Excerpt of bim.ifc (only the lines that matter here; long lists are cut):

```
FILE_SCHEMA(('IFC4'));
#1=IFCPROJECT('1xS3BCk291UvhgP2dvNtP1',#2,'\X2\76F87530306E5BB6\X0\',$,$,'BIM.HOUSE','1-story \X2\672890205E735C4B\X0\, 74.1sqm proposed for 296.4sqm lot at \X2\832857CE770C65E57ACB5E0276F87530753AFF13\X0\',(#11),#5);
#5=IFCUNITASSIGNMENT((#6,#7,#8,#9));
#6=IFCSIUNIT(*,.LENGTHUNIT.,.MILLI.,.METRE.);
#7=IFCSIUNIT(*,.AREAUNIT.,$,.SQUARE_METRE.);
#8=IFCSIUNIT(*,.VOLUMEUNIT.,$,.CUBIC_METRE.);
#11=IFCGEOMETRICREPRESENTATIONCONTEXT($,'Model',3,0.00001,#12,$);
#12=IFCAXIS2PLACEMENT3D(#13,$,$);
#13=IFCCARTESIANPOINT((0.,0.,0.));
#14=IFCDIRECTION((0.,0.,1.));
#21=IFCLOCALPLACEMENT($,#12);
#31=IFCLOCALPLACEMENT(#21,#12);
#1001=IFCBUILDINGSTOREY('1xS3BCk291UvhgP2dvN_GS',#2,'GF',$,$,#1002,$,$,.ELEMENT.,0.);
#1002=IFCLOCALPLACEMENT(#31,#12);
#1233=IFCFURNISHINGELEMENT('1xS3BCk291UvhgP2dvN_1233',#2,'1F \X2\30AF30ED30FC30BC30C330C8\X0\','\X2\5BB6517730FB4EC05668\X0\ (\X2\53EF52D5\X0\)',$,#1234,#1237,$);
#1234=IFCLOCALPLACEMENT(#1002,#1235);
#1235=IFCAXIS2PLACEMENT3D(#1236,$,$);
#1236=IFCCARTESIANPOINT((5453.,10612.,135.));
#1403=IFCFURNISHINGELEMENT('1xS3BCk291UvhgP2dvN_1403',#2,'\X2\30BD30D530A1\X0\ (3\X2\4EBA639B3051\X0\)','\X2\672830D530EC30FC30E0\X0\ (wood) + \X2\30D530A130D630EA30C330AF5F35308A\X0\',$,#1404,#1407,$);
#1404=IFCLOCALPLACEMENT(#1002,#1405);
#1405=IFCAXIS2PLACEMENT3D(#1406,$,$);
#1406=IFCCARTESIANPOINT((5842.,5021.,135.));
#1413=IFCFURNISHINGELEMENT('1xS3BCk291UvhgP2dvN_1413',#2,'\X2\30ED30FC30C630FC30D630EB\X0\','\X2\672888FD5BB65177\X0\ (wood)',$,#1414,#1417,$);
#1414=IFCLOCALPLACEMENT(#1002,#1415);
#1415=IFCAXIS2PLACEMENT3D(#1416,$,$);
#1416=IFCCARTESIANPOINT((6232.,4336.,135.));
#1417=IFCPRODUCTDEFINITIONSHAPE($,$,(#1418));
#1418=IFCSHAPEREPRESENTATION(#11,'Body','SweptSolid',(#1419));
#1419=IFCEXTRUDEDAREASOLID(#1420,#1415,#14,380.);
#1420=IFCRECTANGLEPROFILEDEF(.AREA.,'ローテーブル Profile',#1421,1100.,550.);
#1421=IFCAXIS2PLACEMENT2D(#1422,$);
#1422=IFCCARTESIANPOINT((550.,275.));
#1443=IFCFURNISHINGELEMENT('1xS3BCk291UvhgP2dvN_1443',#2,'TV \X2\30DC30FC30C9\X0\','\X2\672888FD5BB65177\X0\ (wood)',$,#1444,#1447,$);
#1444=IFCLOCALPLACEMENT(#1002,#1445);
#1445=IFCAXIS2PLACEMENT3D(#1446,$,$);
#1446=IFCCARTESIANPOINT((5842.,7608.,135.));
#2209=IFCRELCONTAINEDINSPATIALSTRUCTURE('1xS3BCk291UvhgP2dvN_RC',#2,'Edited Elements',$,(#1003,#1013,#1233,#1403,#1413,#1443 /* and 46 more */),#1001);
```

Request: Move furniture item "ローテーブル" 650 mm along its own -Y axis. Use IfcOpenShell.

```python
import ifcopenshell
import ifcopenshell.api.geometry
import ifcopenshell.util.placement
import ifcopenshell.util.unit

model = ifcopenshell.open("bim.ifc")
unit_scale = ifcopenshell.util.unit.calculate_unit_scale(model)

item = model.by_guid("1xS3BCk291UvhgP2dvN_1413")
matrix = ifcopenshell.util.placement.get_local_placement(item.ObjectPlacement)
matrix[:3, 3] -= matrix[:3, 1] * 0.65 / unit_scale
ifcopenshell.api.geometry.edit_object_placement(model, product=item, matrix=matrix, is_si=False)

print(ifcopenshell.util.placement.get_local_placement(item.ObjectPlacement).round(3) + 0.0)

model.write("bim_v2.ifc")
```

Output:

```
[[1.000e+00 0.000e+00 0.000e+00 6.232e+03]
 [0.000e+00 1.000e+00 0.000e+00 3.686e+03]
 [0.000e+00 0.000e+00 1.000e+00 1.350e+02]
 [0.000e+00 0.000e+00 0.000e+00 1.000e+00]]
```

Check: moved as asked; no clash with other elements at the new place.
